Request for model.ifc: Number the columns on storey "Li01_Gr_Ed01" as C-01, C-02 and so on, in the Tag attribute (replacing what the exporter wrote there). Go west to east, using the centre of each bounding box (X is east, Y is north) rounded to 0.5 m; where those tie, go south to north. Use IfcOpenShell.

First a look at what the model holds.

```python
import ifcopenshell
import ifcopenshell.util.element
import ifcopenshell.util.placement

model = ifcopenshell.open("model.ifc")
print(model.schema)
storey = next(s for s in model.by_type("IfcBuildingStorey") if s.Name == "Li01_Gr_Ed01")
columns = [e for e in ifcopenshell.util.element.get_decomposition(storey) if e.is_a("IfcColumn")]
for e in sorted(columns, key=lambda e: e.id()):
    origin = ifcopenshell.util.placement.get_local_placement(e.ObjectPlacement)[:3, 3]
    print(e.id(), e.Tag, e.Name, origin.round(2) + 0.0, sep=" | ")
```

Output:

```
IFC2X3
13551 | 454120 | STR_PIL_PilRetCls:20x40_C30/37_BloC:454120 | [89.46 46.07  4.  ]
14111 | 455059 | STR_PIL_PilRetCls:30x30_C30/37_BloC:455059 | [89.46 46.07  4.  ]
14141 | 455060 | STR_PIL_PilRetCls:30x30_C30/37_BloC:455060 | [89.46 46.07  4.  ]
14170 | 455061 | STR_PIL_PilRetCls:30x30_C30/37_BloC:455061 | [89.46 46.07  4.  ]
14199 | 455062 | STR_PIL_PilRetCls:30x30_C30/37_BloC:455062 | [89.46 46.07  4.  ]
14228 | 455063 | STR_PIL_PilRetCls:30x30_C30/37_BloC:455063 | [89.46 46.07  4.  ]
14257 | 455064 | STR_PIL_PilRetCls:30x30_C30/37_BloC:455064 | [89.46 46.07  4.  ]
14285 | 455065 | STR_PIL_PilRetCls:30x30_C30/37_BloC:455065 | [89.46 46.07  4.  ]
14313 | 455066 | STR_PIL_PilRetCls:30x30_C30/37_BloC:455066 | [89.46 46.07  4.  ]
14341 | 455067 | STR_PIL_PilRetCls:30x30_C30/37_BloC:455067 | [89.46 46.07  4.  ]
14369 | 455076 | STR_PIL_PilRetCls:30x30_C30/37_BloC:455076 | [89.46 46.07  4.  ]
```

```python
import ifcopenshell
import ifcopenshell.geom
import ifcopenshell.util.element
import ifcopenshell.util.shape

model = ifcopenshell.open("model.ifc")
settings = ifcopenshell.geom.settings()
settings.set("use-world-coords", True)


def centre(element):
    shape = ifcopenshell.geom.create_shape(settings, element)
    return ifcopenshell.util.shape.get_bbox_centroid(shape.geometry)


storey = next(s for s in model.by_type("IfcBuildingStorey") if s.Name == "Li01_Gr_Ed01")
columns = [e for e in ifcopenshell.util.element.get_decomposition(storey) if e.is_a("IfcColumn")]

# Insertion points can sit at a corner or the storey origin, so sort by the geometry (in metres).
centres = {e: centre(e) for e in columns}
columns.sort(key=lambda e: (round(centres[e][0] / 0.5), centres[e][1]))

for i, e in enumerate(columns, start=1):
    number = f"C-{i:02d}"
    e.Tag = number
    print(e.id(), number)

model.write("model_updated.ifc")
```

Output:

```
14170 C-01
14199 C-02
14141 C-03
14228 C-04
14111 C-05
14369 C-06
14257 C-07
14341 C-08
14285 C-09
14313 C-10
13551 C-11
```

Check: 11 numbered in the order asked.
